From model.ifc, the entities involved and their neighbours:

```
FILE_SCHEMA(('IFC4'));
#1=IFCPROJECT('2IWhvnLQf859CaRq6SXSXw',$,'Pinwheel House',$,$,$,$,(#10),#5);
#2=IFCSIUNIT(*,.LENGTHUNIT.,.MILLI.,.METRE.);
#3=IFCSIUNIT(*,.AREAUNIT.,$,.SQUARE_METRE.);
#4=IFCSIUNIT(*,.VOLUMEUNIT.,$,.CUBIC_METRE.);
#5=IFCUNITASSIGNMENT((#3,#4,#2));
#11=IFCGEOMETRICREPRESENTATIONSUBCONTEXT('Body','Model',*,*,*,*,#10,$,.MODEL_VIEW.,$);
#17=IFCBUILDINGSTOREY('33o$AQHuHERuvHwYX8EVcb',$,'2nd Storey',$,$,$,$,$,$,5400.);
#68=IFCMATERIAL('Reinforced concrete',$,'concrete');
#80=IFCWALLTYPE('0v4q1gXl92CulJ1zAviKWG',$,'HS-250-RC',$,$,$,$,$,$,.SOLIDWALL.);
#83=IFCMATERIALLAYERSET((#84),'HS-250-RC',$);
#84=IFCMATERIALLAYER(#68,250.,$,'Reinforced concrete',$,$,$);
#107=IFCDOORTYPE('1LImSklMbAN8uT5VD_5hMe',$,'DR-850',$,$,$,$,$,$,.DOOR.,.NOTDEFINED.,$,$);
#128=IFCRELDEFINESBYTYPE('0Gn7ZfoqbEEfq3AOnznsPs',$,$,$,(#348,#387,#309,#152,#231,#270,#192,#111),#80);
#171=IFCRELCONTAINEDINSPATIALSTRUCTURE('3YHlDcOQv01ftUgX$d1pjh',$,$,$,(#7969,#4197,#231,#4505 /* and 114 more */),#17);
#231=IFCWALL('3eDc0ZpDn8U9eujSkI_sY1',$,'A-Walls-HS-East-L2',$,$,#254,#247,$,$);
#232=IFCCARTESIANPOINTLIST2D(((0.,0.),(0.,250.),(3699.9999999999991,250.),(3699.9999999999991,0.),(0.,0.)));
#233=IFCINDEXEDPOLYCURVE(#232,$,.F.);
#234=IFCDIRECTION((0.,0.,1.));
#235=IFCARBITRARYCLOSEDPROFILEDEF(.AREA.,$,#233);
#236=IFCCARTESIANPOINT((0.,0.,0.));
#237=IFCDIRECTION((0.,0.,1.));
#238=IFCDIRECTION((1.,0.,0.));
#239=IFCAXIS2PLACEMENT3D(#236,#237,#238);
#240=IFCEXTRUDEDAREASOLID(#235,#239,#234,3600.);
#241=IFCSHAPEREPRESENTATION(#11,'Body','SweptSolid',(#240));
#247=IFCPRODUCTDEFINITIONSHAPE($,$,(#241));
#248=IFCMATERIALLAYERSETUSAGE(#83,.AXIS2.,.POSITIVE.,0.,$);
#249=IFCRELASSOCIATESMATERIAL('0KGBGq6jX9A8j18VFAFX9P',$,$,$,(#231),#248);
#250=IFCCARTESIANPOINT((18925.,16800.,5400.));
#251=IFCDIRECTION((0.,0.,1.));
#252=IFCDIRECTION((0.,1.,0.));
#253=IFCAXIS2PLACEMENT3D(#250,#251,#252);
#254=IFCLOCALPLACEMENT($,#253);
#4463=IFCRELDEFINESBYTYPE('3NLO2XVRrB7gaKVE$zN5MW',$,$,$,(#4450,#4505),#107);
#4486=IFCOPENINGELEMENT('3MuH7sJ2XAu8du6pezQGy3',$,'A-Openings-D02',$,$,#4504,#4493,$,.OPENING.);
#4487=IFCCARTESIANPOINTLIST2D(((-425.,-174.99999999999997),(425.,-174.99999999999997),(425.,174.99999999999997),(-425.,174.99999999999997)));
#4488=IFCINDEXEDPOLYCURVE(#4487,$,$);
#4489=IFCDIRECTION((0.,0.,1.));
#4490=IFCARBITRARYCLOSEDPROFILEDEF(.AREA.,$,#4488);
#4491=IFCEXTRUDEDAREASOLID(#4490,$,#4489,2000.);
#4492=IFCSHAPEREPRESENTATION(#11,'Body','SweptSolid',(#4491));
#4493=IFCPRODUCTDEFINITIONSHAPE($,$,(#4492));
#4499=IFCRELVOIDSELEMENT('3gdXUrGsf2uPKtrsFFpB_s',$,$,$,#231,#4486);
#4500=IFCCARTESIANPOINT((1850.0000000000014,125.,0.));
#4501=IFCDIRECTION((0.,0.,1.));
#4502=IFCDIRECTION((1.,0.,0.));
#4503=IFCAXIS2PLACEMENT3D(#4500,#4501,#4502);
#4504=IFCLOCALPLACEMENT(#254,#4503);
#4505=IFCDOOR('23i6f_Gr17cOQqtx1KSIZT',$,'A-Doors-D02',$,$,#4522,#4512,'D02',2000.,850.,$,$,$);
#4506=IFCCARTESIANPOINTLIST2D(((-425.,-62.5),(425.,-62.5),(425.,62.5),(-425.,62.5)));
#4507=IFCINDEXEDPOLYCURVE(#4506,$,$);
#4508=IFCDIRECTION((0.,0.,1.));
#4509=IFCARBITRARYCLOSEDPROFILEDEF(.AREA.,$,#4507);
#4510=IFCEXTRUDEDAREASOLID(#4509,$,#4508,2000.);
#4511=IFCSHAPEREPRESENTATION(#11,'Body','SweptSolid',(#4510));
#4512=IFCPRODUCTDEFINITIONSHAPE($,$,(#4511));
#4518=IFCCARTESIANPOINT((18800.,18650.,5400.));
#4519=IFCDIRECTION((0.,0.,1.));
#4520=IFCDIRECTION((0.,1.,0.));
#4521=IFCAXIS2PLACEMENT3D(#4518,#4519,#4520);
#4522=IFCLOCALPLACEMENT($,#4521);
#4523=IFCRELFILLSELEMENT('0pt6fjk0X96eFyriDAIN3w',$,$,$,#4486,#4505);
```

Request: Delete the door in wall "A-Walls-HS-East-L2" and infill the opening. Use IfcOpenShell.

```python
import ifcopenshell
import ifcopenshell.api.feature
import ifcopenshell.api.root
import ifcopenshell.geom
import ifcopenshell.util.shape

model = ifcopenshell.open("model.ifc")
settings = ifcopenshell.geom.settings()


def volume(element):
    """Net volume in cubic metres, openings subtracted."""
    shape = ifcopenshell.geom.create_shape(settings, element)
    return ifcopenshell.util.shape.get_volume(shape.geometry)


door = model.by_guid("23i6f_Gr17cOQqtx1KSIZT")
opening = door.FillsVoids[0].RelatingOpeningElement
wall = opening.VoidsElements[0].RelatingBuildingElement
before = volume(wall)

ifcopenshell.api.root.remove_product(model, product=door)
ifcopenshell.api.feature.remove_feature(model, feature=opening)

after = volume(wall)

print(f"wall volume {before:.3f} -> {after:.3f} m3")

model.write("model_updated.ifc")
```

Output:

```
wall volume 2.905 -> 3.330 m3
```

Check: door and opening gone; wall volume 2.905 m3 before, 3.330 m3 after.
